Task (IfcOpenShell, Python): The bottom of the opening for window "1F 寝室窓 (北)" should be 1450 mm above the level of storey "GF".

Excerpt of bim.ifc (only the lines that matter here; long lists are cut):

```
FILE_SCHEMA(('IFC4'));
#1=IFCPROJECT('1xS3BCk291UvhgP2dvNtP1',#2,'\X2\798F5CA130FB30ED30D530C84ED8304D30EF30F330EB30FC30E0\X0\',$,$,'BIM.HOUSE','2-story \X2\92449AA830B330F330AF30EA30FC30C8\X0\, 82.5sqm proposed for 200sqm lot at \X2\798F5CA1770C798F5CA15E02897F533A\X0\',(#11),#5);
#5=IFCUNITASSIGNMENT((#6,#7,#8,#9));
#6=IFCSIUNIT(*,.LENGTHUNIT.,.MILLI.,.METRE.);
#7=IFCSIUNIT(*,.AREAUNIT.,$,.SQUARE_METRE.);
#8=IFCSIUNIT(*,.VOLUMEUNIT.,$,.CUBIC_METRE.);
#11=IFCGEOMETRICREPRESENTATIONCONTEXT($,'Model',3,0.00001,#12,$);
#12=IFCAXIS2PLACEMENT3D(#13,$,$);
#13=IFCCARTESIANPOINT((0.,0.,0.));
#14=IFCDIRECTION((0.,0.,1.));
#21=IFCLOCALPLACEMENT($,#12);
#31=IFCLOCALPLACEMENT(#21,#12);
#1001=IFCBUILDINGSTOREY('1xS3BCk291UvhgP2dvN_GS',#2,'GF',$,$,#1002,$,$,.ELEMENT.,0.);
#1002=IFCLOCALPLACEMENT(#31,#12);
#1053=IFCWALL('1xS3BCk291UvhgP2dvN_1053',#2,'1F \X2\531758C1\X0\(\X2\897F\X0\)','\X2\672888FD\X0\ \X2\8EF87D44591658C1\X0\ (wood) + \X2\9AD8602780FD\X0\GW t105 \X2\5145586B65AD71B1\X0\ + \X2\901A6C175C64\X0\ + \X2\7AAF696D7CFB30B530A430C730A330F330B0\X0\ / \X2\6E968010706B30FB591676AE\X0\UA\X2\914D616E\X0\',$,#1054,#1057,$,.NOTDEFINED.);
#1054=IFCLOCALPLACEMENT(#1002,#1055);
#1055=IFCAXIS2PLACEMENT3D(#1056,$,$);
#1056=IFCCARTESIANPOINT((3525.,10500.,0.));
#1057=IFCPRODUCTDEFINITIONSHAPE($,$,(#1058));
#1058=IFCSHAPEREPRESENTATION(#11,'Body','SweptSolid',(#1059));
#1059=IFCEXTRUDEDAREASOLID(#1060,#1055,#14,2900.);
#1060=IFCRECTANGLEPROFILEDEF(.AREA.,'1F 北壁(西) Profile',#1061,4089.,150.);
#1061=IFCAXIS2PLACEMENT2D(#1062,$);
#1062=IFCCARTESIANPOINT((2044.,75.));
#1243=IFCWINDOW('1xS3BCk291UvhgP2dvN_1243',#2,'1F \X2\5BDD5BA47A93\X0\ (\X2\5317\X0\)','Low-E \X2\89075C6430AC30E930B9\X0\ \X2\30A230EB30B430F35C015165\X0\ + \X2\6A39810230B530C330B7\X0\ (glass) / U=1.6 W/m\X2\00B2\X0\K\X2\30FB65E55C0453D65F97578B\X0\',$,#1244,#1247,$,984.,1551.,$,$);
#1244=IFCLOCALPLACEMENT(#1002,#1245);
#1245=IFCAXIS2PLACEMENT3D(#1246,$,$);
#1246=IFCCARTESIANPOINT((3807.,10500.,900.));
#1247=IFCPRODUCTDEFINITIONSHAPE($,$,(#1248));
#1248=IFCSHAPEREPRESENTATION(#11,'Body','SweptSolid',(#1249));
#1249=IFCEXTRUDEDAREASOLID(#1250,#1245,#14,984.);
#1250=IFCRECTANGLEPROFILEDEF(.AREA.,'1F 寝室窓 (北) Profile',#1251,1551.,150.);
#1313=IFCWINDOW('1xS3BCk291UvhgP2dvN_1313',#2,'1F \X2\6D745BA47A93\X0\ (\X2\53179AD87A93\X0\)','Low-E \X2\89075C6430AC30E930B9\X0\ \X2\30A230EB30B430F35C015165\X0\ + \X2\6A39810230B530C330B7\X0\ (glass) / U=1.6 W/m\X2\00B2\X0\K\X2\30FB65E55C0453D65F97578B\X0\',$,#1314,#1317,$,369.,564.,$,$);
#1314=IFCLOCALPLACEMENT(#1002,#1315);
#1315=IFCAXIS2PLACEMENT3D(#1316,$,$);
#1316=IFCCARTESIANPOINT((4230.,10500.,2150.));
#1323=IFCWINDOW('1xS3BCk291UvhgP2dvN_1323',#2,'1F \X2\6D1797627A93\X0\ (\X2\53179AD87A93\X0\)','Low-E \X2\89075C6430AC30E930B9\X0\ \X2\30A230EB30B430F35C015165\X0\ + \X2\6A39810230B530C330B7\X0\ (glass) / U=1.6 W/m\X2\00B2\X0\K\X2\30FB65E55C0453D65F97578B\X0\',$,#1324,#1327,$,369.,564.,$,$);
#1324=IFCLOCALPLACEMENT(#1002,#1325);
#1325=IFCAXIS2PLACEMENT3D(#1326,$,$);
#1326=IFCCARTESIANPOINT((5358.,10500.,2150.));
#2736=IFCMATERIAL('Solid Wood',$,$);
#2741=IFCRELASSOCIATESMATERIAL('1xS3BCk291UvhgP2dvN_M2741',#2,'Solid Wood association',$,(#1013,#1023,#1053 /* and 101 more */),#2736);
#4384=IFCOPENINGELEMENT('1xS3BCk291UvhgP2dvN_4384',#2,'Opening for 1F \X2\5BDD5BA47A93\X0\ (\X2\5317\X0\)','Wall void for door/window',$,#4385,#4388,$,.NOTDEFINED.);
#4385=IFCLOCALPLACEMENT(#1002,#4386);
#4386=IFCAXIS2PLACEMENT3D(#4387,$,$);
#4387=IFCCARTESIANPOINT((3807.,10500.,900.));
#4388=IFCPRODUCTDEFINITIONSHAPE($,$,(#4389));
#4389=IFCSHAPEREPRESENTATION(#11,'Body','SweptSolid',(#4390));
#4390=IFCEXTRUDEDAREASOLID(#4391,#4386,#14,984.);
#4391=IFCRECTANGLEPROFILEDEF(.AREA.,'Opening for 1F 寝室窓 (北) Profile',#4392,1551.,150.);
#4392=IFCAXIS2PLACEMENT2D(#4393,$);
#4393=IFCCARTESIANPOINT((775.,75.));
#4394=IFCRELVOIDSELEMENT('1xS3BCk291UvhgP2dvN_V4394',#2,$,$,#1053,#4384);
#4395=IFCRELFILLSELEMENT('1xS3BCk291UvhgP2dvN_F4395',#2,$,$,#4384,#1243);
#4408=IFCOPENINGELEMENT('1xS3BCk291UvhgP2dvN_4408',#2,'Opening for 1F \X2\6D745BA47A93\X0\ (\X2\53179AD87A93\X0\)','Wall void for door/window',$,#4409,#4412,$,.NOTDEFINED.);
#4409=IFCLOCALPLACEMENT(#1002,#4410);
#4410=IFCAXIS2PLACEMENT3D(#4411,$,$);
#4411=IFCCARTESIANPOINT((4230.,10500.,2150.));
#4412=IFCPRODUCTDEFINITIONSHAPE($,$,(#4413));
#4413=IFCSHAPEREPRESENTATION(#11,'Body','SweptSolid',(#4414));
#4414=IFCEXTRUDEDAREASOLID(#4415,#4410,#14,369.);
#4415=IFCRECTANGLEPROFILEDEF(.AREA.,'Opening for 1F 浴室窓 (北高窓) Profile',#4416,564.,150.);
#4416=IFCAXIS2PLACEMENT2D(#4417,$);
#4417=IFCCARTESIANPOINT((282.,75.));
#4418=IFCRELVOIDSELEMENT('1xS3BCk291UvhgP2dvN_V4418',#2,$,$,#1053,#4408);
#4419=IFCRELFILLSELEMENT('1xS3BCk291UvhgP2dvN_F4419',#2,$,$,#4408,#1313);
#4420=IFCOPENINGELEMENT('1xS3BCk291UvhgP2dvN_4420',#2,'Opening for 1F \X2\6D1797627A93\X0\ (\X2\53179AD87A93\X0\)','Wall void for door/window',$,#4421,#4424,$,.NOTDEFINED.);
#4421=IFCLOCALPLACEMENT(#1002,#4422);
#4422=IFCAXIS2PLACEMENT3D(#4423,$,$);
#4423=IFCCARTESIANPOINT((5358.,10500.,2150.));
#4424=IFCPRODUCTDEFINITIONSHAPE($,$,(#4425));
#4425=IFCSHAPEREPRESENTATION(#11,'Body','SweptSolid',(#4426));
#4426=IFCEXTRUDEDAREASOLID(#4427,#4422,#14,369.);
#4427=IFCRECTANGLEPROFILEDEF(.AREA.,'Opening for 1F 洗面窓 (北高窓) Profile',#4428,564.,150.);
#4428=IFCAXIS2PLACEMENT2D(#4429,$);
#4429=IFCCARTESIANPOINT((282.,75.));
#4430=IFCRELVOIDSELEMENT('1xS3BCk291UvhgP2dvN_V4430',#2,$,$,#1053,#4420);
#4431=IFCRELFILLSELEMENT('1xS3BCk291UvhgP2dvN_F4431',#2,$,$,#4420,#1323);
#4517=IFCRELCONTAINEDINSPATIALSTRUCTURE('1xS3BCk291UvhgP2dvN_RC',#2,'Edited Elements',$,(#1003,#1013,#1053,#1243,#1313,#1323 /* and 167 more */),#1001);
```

```python
import numpy as np
import ifcopenshell
import ifcopenshell.api.geometry
import ifcopenshell.geom
import ifcopenshell.util.element
import ifcopenshell.util.placement
import ifcopenshell.util.shape
import ifcopenshell.util.unit

model = ifcopenshell.open("bim.ifc")
unit_scale = ifcopenshell.util.unit.calculate_unit_scale(model)

window = model.by_id(1243)
opening = window.FillsVoids[0].RelatingOpeningElement
storey = ifcopenshell.util.element.get_container(window, ifc_class="IfcBuildingStorey")
level = ifcopenshell.util.placement.get_local_placement(storey.ObjectPlacement)[2, 3]

# The opening's origin need not be at the sill, so measure its lowest point.
shape = ifcopenshell.geom.create_shape(ifcopenshell.geom.settings(), opening)
bottom = ifcopenshell.util.shape.get_shape_bottom_elevation(shape, shape.geometry) / unit_scale
dz = level + 1.45 / unit_scale - bottom

shift = np.array([0.0, 0.0, dz])
# The window is not placed relative to its opening, so move both.
for product in (opening, window):
    matrix = ifcopenshell.util.placement.get_local_placement(product.ObjectPlacement)
    matrix[:3, 3] += shift
    ifcopenshell.api.geometry.edit_object_placement(model, product=product, matrix=matrix, is_si=False)

print(f"moved by {dz * unit_scale:+.3f} m")

model.write("bim_rev.ifc")
```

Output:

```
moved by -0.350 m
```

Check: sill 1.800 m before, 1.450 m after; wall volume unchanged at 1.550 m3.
